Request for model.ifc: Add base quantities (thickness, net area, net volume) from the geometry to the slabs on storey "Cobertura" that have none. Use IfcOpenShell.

First a look at what the model holds.

```python
import ifcopenshell
import ifcopenshell.util.element
import ifcopenshell.util.unit

model = ifcopenshell.open("model.ifc")
print(model.schema)
for unit_type in ("LENGTHUNIT", "AREAUNIT", "VOLUMEUNIT"):
    print(unit_type, ifcopenshell.util.unit.calculate_unit_scale(model, unit_type))
storey = next(s for s in model.by_type("IfcBuildingStorey") if s.Name == "Cobertura")
slabs = [e for e in ifcopenshell.util.element.get_decomposition(storey) if e.is_a("IfcSlab")]
for e in sorted(slabs, key=lambda e: e.id()):
    print(e.id(), e.is_a(), e.Name, list(ifcopenshell.util.element.get_psets(e, qtos_only=True)), sep=" | ")
```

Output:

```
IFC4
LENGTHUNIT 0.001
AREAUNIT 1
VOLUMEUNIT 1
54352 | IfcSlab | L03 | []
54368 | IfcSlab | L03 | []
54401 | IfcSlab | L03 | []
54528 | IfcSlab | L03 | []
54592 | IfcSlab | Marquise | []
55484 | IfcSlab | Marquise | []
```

```python
import ifcopenshell
import ifcopenshell.api.pset
import ifcopenshell.geom
import ifcopenshell.util.element
import ifcopenshell.util.shape
import ifcopenshell.util.unit

model = ifcopenshell.open("model.ifc")
unit_scale = ifcopenshell.util.unit.calculate_unit_scale(model)
area_scale = ifcopenshell.util.unit.calculate_unit_scale(model, "AREAUNIT")
volume_scale = ifcopenshell.util.unit.calculate_unit_scale(model, "VOLUMEUNIT")
settings = ifcopenshell.geom.settings()

storey = next(s for s in model.by_type("IfcBuildingStorey") if s.Name == "Cobertura")
slabs = [e for e in ifcopenshell.util.element.get_decomposition(storey) if e.is_a("IfcSlab")]

for e in sorted(slabs, key=lambda e: e.id()):
    if ifcopenshell.util.element.get_psets(e, qtos_only=True, should_inherit=False):
        continue
    # Geometry comes back in metres, in the element's own axes.
    shape = ifcopenshell.geom.create_shape(settings, e)
    values = {
        "Width": ifcopenshell.util.shape.get_z(shape.geometry) / unit_scale,
        "NetArea": ifcopenshell.util.shape.get_footprint_area(shape.geometry) / area_scale,
        "NetVolume": ifcopenshell.util.shape.get_volume(shape.geometry) / volume_scale,
    }
    qto = ifcopenshell.api.pset.add_qto(model, product=e, name="Qto_SlabBaseQuantities")
    ifcopenshell.api.pset.edit_qto(model, qto=qto, properties=values)
    print(e.id(), {k: round(v, 3) for k, v in values.items()})

model.write("model_edited.ifc")
```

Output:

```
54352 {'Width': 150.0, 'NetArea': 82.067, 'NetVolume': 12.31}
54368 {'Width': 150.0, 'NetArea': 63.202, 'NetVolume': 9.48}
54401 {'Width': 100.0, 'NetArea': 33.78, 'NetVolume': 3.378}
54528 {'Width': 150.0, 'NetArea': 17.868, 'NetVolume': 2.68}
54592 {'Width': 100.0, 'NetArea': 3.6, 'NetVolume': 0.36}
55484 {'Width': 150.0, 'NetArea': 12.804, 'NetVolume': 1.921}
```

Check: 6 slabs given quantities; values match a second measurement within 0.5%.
